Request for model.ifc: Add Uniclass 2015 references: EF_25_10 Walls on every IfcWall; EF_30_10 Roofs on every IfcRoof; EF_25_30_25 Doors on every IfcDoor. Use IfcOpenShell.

First a look at what the model holds.

```python
import ifcopenshell

model = ifcopenshell.open("model.ifc")
print(model.schema)
print("classifications:", [c.Name for c in model.by_type("IfcClassification")])
for ifc_class in ("IfcDoor", "IfcRoof", "IfcStair", "IfcWall", "IfcWindow"):
    print(ifc_class, len(model.by_type(ifc_class)))
```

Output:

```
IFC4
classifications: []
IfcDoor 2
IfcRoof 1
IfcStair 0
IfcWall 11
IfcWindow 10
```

```python
import ifcopenshell
import ifcopenshell.api.classification

model = ifcopenshell.open("model.ifc")

system = ifcopenshell.api.classification.add_classification(model, classification="Uniclass 2015")

codes = {
    "IfcWall": ("EF_25_10", "Walls"),
    "IfcRoof": ("EF_30_10", "Roofs"),
    "IfcDoor": ("EF_25_30_25", "Doors"),
}
for ifc_class, (code, name) in codes.items():
    products = model.by_type(ifc_class)
    ifcopenshell.api.classification.add_reference(
        model, products=products, classification=system, identification=code, name=name
    )
    print(code, len(products))

model.write("model_rev.ifc")
```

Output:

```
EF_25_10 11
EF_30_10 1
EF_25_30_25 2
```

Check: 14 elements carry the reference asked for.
